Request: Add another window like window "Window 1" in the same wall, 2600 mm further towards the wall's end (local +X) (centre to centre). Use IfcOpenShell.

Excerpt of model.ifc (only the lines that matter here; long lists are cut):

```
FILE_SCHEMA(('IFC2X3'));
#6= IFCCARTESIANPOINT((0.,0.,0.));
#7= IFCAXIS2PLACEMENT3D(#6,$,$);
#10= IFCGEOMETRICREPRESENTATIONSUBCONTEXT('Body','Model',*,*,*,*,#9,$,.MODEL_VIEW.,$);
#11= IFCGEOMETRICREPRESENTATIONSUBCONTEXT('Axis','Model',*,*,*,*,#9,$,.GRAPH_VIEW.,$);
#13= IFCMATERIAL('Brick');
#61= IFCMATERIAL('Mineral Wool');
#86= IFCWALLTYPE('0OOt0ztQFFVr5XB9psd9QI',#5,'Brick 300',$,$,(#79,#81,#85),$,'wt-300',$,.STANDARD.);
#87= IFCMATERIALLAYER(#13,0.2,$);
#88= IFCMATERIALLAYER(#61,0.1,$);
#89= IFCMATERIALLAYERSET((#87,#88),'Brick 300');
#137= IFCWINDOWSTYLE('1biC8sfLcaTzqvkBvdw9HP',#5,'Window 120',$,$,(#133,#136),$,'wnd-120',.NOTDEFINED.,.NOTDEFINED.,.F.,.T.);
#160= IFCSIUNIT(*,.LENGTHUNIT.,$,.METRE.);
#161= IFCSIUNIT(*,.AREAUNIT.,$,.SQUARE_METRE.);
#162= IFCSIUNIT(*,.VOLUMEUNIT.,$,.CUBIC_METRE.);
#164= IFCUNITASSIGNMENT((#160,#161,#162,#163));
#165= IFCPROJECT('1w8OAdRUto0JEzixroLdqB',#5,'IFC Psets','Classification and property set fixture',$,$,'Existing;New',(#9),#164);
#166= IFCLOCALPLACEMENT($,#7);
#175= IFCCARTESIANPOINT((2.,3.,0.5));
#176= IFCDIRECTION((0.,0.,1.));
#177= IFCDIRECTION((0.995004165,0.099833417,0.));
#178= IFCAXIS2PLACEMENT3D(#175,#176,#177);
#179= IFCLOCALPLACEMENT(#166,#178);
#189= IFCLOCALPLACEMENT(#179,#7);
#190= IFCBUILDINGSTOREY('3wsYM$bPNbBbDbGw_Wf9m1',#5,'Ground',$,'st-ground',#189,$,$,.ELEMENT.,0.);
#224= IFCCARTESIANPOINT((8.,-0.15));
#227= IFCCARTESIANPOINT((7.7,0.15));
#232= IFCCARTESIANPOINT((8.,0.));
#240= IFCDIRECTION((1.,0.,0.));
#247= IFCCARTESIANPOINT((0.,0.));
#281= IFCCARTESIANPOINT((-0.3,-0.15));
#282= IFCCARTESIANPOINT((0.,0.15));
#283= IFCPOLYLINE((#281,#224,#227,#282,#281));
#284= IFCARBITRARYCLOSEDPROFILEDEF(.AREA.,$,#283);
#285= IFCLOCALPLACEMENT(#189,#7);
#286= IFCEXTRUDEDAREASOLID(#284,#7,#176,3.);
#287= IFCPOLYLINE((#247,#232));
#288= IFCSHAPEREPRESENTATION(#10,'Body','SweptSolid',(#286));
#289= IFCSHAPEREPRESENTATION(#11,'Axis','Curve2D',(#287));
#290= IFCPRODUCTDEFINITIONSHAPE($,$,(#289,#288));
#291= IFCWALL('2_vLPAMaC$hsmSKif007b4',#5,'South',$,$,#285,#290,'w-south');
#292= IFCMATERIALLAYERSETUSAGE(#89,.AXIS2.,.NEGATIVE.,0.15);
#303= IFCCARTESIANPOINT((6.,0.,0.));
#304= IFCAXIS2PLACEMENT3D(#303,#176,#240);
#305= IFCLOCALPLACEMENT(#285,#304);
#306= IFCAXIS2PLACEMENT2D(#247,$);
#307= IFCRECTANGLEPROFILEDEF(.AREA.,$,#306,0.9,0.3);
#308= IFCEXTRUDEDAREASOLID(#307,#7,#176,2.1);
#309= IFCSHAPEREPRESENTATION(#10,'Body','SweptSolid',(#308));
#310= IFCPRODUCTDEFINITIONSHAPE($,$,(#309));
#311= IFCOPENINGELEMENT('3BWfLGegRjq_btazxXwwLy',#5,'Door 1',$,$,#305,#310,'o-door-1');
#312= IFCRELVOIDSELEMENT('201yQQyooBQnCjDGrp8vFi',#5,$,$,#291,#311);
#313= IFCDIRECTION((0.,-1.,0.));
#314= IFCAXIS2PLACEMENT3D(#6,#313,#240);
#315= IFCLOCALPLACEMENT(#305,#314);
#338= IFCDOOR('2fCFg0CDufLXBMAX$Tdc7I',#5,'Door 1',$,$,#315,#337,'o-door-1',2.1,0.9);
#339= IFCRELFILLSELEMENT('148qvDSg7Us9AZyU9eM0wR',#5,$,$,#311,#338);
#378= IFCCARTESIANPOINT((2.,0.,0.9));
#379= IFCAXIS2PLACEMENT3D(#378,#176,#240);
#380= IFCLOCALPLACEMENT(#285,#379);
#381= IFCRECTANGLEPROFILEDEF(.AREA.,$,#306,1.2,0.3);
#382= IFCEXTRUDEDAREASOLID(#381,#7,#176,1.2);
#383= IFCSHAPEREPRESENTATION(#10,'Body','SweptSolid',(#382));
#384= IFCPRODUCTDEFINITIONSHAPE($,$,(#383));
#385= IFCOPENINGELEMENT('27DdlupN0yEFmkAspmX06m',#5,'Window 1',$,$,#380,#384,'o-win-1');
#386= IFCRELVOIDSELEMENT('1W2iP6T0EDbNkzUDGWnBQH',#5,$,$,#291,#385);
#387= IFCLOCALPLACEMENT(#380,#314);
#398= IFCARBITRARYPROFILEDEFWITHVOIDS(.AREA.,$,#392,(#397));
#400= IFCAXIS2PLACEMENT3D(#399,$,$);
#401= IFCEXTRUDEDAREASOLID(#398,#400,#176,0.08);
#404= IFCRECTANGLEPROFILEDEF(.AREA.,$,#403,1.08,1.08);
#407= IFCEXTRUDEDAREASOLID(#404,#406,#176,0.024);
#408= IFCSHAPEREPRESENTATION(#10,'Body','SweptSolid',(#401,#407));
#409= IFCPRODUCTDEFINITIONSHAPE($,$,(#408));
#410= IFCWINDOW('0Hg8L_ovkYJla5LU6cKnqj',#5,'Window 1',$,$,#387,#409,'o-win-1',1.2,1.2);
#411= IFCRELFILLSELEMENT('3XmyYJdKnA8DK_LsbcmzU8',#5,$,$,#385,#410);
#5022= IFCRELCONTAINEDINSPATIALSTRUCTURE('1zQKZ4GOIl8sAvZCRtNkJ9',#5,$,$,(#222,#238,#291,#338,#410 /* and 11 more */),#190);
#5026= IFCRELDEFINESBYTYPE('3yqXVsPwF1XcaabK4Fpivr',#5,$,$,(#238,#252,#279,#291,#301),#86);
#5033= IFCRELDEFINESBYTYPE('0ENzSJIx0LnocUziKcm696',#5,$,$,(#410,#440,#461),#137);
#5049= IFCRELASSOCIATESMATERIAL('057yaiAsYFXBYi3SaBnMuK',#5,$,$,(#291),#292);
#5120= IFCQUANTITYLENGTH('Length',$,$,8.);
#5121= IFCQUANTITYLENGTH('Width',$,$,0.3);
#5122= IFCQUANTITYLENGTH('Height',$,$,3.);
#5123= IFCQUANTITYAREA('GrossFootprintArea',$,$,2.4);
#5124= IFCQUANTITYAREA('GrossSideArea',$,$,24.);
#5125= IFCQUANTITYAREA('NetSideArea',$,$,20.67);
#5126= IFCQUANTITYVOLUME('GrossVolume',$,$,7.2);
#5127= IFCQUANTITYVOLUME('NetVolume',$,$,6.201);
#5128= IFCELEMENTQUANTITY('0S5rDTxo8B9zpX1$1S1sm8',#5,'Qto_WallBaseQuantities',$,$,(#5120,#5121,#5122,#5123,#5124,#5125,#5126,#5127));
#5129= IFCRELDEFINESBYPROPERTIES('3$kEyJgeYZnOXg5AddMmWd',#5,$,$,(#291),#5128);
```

```python
import ifcopenshell
import ifcopenshell.api.feature
import ifcopenshell.api.geometry
import ifcopenshell.api.pset
import ifcopenshell.api.root
import ifcopenshell.geom
import ifcopenshell.util.element
import ifcopenshell.util.placement
import ifcopenshell.util.shape
import ifcopenshell.util.unit

model = ifcopenshell.open("model.ifc")
unit_scale = ifcopenshell.util.unit.calculate_unit_scale(model)
area_scale = ifcopenshell.util.unit.calculate_unit_scale(model, "AREAUNIT")
volume_scale = ifcopenshell.util.unit.calculate_unit_scale(model, "VOLUMEUNIT")
settings = ifcopenshell.geom.settings()


def volume(element):
    """Net volume in cubic metres, openings subtracted."""
    shape = ifcopenshell.geom.create_shape(settings, element)
    return ifcopenshell.util.shape.get_volume(shape.geometry)


def reuse_history(source, copy):
    """copy_class also copies each property set's owner history, people and application; keep the originals."""
    for rel in copy.IsDefinedBy:
        if rel.is_a("IfcRelDefinesByProperties") and (history := rel.RelatingPropertyDefinition.OwnerHistory):
            rel.RelatingPropertyDefinition.OwnerHistory = source.OwnerHistory
            ifcopenshell.util.element.remove_deep2(model, history)


window = model.by_id(410)
opening = window.FillsVoids[0].RelatingOpeningElement
wall = opening.VoidsElements[0].RelatingBuildingElement
before = volume(wall)
shift = ifcopenshell.util.placement.get_local_placement(wall.ObjectPlacement)[:3, 0] * 2.6 / unit_scale

# copy_class copies the void relationship, type, container and properties, but no geometry.
new_opening = ifcopenshell.api.root.copy_class(model, product=opening)
new_opening.Representation = ifcopenshell.util.element.copy_deep(
    model, opening.Representation, exclude=["IfcGeometricRepresentationContext", "IfcRepresentationMap"]
)
new_opening.Tag = None
new_window = ifcopenshell.api.root.copy_class(model, product=window)
new_window.Representation = ifcopenshell.util.element.copy_deep(
    model, window.Representation, exclude=["IfcGeometricRepresentationContext", "IfcRepresentationMap"]
)
new_window.Tag = None
reuse_history(window, new_window)
fills = ifcopenshell.api.feature.add_filling(model, opening=new_opening, element=new_window)
fills.OwnerHistory = new_window.OwnerHistory  # required in IFC2X3

for old, new in ((opening, new_opening), (window, new_window)):
    matrix = ifcopenshell.util.placement.get_local_placement(old.ObjectPlacement)
    matrix[:3, 3] += shift
    ifcopenshell.api.geometry.edit_object_placement(model, product=new, matrix=matrix, is_si=False)

after = volume(wall)
thickness = 0.3  # wall thickness in metres

# Update the wall's stored quantities.
qto = model.by_id(ifcopenshell.util.element.get_pset(wall, "Qto_WallBaseQuantities", should_inherit=False)["id"])
ifcopenshell.api.pset.edit_qto(model, qto=qto, properties={
    "NetSideArea": after / thickness / area_scale,
    "NetVolume": after / volume_scale,
})

print(f"wall volume {before:.3f} -> {after:.3f} m3")

model.write("model-out.ifc")
```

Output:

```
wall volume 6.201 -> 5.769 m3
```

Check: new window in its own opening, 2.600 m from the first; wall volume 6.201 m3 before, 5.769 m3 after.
